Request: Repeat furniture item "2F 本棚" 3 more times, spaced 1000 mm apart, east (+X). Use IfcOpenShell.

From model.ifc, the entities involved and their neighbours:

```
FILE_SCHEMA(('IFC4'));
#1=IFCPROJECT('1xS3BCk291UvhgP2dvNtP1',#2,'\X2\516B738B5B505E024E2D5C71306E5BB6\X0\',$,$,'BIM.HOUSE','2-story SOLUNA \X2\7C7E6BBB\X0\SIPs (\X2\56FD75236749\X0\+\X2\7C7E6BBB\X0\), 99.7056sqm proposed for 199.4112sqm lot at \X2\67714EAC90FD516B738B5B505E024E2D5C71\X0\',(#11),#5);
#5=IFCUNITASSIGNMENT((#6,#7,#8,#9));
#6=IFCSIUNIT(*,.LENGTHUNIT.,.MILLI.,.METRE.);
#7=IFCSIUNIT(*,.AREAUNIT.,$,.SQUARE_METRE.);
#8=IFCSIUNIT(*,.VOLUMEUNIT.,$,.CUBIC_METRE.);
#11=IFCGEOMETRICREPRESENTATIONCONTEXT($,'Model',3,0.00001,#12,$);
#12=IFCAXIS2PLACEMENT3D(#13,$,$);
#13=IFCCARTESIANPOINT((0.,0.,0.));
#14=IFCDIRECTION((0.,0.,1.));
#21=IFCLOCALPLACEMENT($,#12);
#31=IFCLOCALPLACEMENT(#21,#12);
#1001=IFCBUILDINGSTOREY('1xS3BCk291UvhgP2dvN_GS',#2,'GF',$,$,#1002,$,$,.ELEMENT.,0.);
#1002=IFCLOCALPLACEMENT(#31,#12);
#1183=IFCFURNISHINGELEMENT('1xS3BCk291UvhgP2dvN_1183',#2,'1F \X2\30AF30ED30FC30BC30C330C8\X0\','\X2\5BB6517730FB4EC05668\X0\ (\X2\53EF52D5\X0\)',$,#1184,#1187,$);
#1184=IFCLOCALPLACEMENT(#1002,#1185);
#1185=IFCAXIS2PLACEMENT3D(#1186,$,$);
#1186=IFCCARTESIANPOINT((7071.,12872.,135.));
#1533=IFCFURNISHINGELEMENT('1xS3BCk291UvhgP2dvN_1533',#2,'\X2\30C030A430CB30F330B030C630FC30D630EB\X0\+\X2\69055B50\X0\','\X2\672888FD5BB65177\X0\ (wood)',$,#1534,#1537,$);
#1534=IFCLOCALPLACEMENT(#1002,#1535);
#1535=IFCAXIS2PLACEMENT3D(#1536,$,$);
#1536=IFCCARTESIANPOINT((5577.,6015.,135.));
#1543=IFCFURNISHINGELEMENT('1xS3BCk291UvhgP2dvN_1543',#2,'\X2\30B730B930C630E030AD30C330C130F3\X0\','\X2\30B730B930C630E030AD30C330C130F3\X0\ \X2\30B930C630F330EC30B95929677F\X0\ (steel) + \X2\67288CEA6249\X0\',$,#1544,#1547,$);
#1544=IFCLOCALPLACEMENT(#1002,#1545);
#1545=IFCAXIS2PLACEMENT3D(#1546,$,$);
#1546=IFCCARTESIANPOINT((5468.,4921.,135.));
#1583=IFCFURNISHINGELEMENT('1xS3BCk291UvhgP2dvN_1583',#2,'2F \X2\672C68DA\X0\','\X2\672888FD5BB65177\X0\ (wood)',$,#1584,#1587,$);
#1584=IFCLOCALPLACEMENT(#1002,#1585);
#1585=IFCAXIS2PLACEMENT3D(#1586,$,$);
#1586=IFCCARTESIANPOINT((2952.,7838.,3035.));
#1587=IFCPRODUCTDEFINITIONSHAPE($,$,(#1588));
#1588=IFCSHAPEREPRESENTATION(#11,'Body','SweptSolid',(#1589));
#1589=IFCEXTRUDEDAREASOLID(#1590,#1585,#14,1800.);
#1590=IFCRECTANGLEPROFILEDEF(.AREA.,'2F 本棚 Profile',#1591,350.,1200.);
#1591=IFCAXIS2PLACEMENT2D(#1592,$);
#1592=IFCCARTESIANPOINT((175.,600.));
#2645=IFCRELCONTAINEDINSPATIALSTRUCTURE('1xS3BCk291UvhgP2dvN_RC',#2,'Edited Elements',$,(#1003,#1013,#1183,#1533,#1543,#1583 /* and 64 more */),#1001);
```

```python
import numpy as np
import ifcopenshell
import ifcopenshell.api.geometry
import ifcopenshell.api.root
import ifcopenshell.util.element
import ifcopenshell.util.placement

model = ifcopenshell.open("model.ifc")


def reuse_history(source, copy):
    """copy_class also copies each property set's owner history, people and application; keep the originals."""
    for rel in copy.IsDefinedBy:
        if rel.is_a("IfcRelDefinesByProperties") and (history := rel.RelatingPropertyDefinition.OwnerHistory):
            rel.RelatingPropertyDefinition.OwnerHistory = source.OwnerHistory
            ifcopenshell.util.element.remove_deep2(model, history)


source = model.by_guid("1xS3BCk291UvhgP2dvN_1583")
base = ifcopenshell.util.placement.get_local_placement(source.ObjectPlacement)
step = np.array([1.0, 0.0, 0.0]) * 1000.0

for i in range(1, 4):
    copy = ifcopenshell.api.root.copy_class(model, product=source)
    copy.Representation = ifcopenshell.util.element.copy_deep(
        model, source.Representation, exclude=["IfcGeometricRepresentationContext", "IfcRepresentationMap"]
    )
    reuse_history(source, copy)
    matrix = base.copy()
    matrix[:3, 3] += i * step
    print("added at", matrix[:3, 3].round(3) + 0.0)
    ifcopenshell.api.geometry.edit_object_placement(model, product=copy, matrix=matrix, is_si=False)

model.write("model_edited.ifc")
```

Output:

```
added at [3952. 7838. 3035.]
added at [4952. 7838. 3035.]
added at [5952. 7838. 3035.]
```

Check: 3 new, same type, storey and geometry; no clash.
